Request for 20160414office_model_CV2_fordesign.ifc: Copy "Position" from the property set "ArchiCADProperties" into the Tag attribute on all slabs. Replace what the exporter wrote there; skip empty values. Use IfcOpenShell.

First a look at what the model holds.

```python
import ifcopenshell
import ifcopenshell.util.element

model = ifcopenshell.open("20160414office_model_CV2_fordesign.ifc")
print(model.schema)
slabs = model.by_type("IfcSlab")
print(len(slabs), "slabs")
for e in slabs[:8]:
    source = ifcopenshell.util.element.get_pset(e, "ArchiCADProperties", "Position")
    target = e.Tag
    print(e.id(), repr(source), repr(target), sep=" | ")
```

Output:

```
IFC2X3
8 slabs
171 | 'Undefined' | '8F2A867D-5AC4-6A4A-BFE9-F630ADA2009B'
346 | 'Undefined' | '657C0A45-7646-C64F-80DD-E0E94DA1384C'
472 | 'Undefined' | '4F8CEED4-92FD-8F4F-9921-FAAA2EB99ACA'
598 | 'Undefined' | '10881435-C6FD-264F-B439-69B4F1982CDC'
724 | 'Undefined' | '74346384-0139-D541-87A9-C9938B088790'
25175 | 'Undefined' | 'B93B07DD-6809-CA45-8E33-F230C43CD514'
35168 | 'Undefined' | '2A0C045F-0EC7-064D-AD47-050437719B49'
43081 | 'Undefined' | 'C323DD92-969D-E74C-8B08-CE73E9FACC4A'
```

```python
import ifcopenshell
import ifcopenshell.util.element

model = ifcopenshell.open("20160414office_model_CV2_fordesign.ifc")

count = 0
for e in model.by_type("IfcSlab"):
    value = ifcopenshell.util.element.get_pset(e, "ArchiCADProperties", "Position")
    current = e.Tag
    if not value or not value.strip() or current == value:
        continue
    e.Tag = value
    count += 1

print(count, "slabs updated")

model.write("20160414office_model_CV2_fordesign_edited.ifc")
```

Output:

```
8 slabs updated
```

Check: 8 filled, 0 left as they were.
